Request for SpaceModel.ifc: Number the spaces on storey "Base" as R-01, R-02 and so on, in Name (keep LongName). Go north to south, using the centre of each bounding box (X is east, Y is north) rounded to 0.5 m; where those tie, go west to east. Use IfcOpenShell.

First a look at what the model holds.

```python
import ifcopenshell
import ifcopenshell.util.element
import ifcopenshell.util.placement

model = ifcopenshell.open("SpaceModel.ifc")
print(model.schema)
storey = next(s for s in model.by_type("IfcBuildingStorey") if s.Name == "Base")
spaces = [e for e in ifcopenshell.util.element.get_decomposition(storey) if e.is_a("IfcSpace")]
for e in sorted(spaces, key=lambda e: e.id()):
    origin = ifcopenshell.util.placement.get_local_placement(e.ObjectPlacement)[:3, 3]
    print(e.id(), e.Name, e.LongName, origin.round(2) + 0.0, sep=" | ")
```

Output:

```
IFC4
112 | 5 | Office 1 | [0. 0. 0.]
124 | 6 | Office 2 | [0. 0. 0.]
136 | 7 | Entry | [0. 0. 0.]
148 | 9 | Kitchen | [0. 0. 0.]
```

```python
import ifcopenshell
import ifcopenshell.geom
import ifcopenshell.util.element
import ifcopenshell.util.shape

model = ifcopenshell.open("SpaceModel.ifc")
settings = ifcopenshell.geom.settings()
settings.set("use-world-coords", True)


def centre(element):
    shape = ifcopenshell.geom.create_shape(settings, element)
    return ifcopenshell.util.shape.get_bbox_centroid(shape.geometry)


storey = next(s for s in model.by_type("IfcBuildingStorey") if s.Name == "Base")
spaces = [e for e in ifcopenshell.util.element.get_decomposition(storey) if e.is_a("IfcSpace")]

# Insertion points can sit at a corner or the storey origin, so sort by the geometry (in metres).
centres = {e: centre(e) for e in spaces}
spaces.sort(key=lambda e: (-round(centres[e][1] / 0.5), centres[e][0]))

for i, e in enumerate(spaces, start=1):
    number = f"R-{i:02d}"
    e.Name = number
    print(e.id(), number)

model.write("SpaceModel_updated.ifc")
```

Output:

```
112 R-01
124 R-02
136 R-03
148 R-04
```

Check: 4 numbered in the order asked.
